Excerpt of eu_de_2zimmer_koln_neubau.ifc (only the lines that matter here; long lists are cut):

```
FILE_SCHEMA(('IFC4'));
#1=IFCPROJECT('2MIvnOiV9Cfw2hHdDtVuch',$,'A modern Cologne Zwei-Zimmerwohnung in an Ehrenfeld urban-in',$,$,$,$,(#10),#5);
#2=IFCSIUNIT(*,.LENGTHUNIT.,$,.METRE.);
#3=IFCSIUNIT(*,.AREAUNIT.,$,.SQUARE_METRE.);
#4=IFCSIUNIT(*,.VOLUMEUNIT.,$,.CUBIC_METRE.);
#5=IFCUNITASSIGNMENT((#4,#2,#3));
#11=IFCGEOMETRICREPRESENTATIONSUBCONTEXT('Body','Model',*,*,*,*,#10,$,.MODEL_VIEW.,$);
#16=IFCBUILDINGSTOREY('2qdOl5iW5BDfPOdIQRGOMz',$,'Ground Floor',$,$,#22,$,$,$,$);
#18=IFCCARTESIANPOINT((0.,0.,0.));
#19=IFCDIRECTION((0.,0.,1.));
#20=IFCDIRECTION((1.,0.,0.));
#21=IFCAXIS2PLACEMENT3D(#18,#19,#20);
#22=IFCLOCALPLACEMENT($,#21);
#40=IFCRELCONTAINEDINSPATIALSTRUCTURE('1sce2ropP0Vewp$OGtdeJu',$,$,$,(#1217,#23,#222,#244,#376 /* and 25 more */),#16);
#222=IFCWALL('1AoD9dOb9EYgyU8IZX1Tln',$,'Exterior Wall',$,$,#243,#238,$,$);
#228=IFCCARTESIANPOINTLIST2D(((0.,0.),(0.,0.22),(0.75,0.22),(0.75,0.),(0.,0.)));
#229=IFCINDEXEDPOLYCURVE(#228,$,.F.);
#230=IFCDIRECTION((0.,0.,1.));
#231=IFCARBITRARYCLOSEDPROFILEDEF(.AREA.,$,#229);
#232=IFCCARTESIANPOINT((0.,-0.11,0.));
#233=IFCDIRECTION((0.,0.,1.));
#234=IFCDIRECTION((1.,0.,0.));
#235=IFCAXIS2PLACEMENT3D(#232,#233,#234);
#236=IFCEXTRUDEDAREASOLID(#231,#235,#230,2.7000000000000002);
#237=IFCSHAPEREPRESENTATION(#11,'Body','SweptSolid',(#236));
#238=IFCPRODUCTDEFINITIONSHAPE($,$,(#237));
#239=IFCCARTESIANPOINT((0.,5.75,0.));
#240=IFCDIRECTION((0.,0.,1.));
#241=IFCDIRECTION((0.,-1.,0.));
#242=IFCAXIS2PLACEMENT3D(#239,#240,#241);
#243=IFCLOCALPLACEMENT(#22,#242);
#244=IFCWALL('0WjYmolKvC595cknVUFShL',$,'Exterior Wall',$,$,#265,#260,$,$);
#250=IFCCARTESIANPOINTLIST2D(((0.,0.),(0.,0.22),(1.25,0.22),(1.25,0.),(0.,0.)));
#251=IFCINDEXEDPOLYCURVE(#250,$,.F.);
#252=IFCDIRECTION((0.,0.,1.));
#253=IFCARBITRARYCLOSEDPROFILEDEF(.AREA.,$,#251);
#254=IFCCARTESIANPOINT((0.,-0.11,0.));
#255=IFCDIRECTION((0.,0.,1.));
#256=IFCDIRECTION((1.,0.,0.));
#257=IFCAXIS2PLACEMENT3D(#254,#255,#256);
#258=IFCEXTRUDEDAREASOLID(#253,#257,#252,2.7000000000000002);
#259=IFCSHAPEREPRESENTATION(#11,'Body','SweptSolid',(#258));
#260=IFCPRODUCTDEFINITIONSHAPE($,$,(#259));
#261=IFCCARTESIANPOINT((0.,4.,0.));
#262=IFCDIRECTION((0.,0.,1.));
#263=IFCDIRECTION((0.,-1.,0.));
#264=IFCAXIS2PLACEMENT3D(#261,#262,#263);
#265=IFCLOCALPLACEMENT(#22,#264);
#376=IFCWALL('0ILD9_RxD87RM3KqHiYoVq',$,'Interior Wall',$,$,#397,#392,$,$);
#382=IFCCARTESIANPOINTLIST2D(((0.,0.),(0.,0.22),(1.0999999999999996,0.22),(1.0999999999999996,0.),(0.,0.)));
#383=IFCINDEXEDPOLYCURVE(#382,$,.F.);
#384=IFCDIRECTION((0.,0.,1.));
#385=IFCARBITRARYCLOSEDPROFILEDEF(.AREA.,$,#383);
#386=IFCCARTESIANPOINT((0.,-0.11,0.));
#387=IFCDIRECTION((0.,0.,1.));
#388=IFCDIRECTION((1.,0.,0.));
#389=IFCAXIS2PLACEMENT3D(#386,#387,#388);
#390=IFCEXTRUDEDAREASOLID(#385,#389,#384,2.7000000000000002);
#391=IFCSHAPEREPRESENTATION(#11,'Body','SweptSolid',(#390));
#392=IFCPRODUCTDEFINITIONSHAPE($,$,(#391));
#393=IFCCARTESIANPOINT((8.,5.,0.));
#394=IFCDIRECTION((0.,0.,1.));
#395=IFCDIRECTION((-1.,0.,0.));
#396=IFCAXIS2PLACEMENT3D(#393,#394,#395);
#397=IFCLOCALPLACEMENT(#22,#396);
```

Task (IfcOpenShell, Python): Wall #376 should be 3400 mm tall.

```python
import ifcopenshell
import ifcopenshell.geom
import ifcopenshell.util.representation
import ifcopenshell.util.shape
import ifcopenshell.util.unit

model = ifcopenshell.open("eu_de_2zimmer_koln_neubau.ifc")
unit_scale = ifcopenshell.util.unit.calculate_unit_scale(model)
settings = ifcopenshell.geom.settings()


def volume(element):
    """Net volume in cubic metres, openings subtracted."""
    shape = ifcopenshell.geom.create_shape(settings, element)
    return ifcopenshell.util.shape.get_volume(shape.geometry)


wall = model.by_guid("0ILD9_RxD87RM3KqHiYoVq")
before = volume(wall)

body = ifcopenshell.util.representation.get_representation(wall, "Model", "Body")
solid = body.Items[0]
old_height = solid.Depth
solid.Depth = 3.4 / unit_scale
after = volume(wall)

print(f"height {old_height:g} -> {solid.Depth:g}, volume {before:.3f} -> {after:.3f} m3")

model.write("eu_de_2zimmer_koln_neubau-out.ifc")
```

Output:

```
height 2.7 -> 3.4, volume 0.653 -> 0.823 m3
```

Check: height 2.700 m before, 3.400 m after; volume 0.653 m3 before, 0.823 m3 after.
